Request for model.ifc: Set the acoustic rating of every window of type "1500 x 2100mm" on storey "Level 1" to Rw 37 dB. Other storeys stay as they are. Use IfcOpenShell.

First a look at what the model holds.

```python
import ifcopenshell
import ifcopenshell.util.element

model = ifcopenshell.open("model.ifc")
print(model.schema)
storey = next(s for s in model.by_type("IfcBuildingStorey") if s.Name == "Level 1")
windows = [e for e in ifcopenshell.util.element.get_decomposition(storey) if e.is_a("IfcWindow")]
seen = {}
for e in windows:
    element_type = ifcopenshell.util.element.get_type(e)
    key = (element_type.Name if element_type != e and element_type else None, ifcopenshell.util.element.get_pset(e, "Pset_WindowCommon", "AcousticRating"))
    seen[key] = seen.get(key, 0) + 1
for (name, value), count in sorted(seen.items(), key=str):
    print(count, "x", name, "|", value)
```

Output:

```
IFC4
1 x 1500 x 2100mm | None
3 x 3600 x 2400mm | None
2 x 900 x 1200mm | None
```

```python
import ifcopenshell
import ifcopenshell.api.pset
import ifcopenshell.util.element

model = ifcopenshell.open("model.ifc")

storey = next(s for s in model.by_type("IfcBuildingStorey") if s.Name == "Level 1")
windows = [e for e in ifcopenshell.util.element.get_decomposition(storey) if e.is_a("IfcWindow")]

count = 0
for e in windows:
    element_type = ifcopenshell.util.element.get_type(e)
    if element_type in (None, e) or element_type.Name != "1500 x 2100mm":
        continue
    # add_pset returns the element's existing set when there is one.
    pset = ifcopenshell.api.pset.add_pset(model, product=e, name="Pset_WindowCommon")
    ifcopenshell.api.pset.edit_pset(model, pset=pset, properties={"AcousticRating": "Rw 37 dB"})
    count += 1

print(count, "windows updated")

model.write("model_v2.ifc")
```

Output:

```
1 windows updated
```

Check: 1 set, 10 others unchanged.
